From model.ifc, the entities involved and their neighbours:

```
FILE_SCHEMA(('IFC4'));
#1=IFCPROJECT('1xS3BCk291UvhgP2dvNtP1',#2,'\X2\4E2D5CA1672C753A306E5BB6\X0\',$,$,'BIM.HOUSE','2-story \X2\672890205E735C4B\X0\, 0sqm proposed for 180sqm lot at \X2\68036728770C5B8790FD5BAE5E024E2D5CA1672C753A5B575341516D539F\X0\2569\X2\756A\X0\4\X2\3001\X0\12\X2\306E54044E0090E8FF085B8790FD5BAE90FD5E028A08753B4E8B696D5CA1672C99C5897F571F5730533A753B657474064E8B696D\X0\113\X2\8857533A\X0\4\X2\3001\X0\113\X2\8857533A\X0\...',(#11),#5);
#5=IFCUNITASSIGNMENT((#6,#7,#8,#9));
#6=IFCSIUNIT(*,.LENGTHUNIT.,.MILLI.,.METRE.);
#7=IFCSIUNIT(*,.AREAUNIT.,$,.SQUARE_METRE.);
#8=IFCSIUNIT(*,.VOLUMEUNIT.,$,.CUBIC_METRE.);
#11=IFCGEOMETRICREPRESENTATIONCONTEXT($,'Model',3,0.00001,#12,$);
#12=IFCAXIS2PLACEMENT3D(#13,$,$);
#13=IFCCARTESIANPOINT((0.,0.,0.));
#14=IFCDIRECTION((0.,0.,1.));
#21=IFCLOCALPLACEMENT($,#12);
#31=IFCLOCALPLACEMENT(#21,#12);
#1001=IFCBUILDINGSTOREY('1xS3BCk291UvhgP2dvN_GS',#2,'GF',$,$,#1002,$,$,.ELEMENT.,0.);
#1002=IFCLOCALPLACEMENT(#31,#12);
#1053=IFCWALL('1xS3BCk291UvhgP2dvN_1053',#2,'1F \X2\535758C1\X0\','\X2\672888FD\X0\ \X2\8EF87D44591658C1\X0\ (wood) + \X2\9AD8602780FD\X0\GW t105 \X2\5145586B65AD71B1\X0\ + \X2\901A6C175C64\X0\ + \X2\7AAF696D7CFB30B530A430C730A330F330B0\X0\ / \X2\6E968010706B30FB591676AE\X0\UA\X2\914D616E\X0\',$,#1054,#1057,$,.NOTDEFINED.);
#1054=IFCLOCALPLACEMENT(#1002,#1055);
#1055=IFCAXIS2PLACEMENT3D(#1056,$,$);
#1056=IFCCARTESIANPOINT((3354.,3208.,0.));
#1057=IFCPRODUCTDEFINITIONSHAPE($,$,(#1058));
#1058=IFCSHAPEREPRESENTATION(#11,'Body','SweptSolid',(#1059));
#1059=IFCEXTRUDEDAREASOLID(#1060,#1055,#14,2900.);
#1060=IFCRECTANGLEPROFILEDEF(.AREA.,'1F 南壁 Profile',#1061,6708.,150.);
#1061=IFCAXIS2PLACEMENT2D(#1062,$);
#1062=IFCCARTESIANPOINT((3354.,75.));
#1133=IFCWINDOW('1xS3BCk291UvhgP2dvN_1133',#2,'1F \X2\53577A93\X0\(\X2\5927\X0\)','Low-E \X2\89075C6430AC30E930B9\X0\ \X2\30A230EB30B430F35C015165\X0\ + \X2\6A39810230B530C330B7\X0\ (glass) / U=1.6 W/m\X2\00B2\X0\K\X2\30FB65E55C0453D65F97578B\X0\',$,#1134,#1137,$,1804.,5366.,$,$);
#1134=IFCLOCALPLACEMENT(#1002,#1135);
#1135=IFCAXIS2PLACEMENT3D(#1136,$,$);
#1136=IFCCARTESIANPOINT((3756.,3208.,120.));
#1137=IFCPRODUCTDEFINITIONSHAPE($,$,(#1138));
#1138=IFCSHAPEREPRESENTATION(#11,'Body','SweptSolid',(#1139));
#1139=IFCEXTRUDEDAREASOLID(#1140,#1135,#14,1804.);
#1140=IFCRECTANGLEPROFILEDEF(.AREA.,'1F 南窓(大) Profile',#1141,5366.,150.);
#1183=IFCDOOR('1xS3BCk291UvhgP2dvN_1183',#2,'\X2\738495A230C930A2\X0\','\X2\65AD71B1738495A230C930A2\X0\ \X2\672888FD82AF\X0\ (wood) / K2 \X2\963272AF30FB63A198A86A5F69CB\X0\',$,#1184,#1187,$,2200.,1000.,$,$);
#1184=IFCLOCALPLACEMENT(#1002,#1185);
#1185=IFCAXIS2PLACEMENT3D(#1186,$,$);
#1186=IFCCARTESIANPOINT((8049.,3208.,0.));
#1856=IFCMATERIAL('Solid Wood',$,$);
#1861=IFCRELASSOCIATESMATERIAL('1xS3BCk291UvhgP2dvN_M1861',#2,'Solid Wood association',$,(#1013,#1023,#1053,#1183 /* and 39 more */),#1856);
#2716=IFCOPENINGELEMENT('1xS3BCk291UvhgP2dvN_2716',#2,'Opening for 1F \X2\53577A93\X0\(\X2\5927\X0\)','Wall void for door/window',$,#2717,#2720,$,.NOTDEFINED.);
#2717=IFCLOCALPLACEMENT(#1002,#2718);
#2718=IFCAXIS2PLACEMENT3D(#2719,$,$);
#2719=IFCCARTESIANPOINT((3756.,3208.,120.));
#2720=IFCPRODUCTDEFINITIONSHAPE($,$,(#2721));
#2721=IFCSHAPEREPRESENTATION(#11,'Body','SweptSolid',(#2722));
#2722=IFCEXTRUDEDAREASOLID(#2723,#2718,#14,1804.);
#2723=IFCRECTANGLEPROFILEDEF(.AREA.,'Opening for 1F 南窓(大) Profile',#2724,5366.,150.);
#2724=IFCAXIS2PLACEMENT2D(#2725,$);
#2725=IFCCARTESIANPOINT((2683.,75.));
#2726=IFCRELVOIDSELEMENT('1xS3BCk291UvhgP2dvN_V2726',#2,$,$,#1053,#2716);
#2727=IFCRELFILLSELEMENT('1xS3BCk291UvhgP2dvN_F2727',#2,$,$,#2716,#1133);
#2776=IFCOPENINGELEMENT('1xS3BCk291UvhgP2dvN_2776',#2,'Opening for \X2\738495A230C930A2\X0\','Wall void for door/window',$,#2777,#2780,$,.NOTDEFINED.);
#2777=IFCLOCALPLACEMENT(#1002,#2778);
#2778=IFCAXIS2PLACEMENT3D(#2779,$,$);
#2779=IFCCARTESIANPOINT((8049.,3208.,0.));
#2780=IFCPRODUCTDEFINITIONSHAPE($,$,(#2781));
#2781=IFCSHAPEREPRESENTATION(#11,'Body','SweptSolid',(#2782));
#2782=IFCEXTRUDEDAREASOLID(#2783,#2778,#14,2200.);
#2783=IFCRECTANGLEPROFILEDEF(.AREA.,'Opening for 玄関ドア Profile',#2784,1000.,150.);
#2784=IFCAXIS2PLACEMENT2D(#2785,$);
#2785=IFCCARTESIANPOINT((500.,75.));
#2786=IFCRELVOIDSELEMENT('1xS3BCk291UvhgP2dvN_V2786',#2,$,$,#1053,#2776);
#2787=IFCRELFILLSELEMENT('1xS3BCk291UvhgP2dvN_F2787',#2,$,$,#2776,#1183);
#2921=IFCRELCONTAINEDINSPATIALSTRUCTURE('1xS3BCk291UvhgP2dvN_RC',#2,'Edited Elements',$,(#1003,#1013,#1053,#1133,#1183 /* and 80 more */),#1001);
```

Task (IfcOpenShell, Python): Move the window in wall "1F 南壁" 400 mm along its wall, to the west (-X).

```python
import ifcopenshell
import ifcopenshell.api.geometry
import ifcopenshell.util.placement
import ifcopenshell.util.unit

model = ifcopenshell.open("model.ifc")
unit_scale = ifcopenshell.util.unit.calculate_unit_scale(model)

window = model.by_id(1133)
opening = window.FillsVoids[0].RelatingOpeningElement
wall = opening.VoidsElements[0].RelatingBuildingElement

wall_matrix = ifcopenshell.util.placement.get_local_placement(wall.ObjectPlacement)
shift = wall_matrix[:3, 0] * -0.4 / unit_scale
before = ifcopenshell.util.placement.get_local_placement(window.ObjectPlacement)[:3, 3].copy()

# The window is not placed relative to its opening, so move both.
for product in (opening, window):
    matrix = ifcopenshell.util.placement.get_local_placement(product.ObjectPlacement)
    matrix[:3, 3] += shift
    ifcopenshell.api.geometry.edit_object_placement(model, product=product, matrix=matrix, is_si=False)

after = ifcopenshell.util.placement.get_local_placement(window.ObjectPlacement)[:3, 3]
print("window moved by", (after - before).round(3) + 0.0)

model.write("model_edited.ifc")
```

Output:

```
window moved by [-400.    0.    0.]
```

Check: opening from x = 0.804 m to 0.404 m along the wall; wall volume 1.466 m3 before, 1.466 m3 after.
